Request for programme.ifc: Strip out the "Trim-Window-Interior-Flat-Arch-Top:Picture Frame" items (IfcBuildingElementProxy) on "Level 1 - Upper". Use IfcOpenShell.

First a look at what the model holds.

```python
import ifcopenshell
import ifcopenshell.util.element

model = ifcopenshell.open("programme.ifc")
print(model.schema)
storey = next(s for s in model.by_type("IfcBuildingStorey") if s.Name == "Level 1 - Upper")
proxies = [e for e in ifcopenshell.util.element.get_decomposition(storey) if e.is_a("IfcBuildingElementProxy")]
seen = {}
for e in proxies:
    element_type = ifcopenshell.util.element.get_type(e)
    name = element_type.Name if element_type not in (None, e) else None
    seen[name] = seen.get(name, 0) + 1
for name, count in sorted(seen.items(), key=str):
    print(count, "x", name)
```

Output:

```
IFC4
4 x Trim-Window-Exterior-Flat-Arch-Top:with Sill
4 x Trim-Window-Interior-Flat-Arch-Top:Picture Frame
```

```python
import ifcopenshell
import ifcopenshell.api.root
import ifcopenshell.util.element

model = ifcopenshell.open("programme.ifc")

storey = next(s for s in model.by_type("IfcBuildingStorey") if s.Name == "Level 1 - Upper")
proxies = [e for e in ifcopenshell.util.element.get_decomposition(storey) if e.is_a("IfcBuildingElementProxy")]
targets = [e for e in proxies if (t := ifcopenshell.util.element.get_type(e)) not in (None, e) and t.Name == "Trim-Window-Interior-Flat-Arch-Top:Picture Frame"]

for e in targets:
    ifcopenshell.api.root.remove_product(model, product=e)
print(len(targets), "removed")

model.write("programme_rev.ifc")
```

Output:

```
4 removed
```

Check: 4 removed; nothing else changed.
